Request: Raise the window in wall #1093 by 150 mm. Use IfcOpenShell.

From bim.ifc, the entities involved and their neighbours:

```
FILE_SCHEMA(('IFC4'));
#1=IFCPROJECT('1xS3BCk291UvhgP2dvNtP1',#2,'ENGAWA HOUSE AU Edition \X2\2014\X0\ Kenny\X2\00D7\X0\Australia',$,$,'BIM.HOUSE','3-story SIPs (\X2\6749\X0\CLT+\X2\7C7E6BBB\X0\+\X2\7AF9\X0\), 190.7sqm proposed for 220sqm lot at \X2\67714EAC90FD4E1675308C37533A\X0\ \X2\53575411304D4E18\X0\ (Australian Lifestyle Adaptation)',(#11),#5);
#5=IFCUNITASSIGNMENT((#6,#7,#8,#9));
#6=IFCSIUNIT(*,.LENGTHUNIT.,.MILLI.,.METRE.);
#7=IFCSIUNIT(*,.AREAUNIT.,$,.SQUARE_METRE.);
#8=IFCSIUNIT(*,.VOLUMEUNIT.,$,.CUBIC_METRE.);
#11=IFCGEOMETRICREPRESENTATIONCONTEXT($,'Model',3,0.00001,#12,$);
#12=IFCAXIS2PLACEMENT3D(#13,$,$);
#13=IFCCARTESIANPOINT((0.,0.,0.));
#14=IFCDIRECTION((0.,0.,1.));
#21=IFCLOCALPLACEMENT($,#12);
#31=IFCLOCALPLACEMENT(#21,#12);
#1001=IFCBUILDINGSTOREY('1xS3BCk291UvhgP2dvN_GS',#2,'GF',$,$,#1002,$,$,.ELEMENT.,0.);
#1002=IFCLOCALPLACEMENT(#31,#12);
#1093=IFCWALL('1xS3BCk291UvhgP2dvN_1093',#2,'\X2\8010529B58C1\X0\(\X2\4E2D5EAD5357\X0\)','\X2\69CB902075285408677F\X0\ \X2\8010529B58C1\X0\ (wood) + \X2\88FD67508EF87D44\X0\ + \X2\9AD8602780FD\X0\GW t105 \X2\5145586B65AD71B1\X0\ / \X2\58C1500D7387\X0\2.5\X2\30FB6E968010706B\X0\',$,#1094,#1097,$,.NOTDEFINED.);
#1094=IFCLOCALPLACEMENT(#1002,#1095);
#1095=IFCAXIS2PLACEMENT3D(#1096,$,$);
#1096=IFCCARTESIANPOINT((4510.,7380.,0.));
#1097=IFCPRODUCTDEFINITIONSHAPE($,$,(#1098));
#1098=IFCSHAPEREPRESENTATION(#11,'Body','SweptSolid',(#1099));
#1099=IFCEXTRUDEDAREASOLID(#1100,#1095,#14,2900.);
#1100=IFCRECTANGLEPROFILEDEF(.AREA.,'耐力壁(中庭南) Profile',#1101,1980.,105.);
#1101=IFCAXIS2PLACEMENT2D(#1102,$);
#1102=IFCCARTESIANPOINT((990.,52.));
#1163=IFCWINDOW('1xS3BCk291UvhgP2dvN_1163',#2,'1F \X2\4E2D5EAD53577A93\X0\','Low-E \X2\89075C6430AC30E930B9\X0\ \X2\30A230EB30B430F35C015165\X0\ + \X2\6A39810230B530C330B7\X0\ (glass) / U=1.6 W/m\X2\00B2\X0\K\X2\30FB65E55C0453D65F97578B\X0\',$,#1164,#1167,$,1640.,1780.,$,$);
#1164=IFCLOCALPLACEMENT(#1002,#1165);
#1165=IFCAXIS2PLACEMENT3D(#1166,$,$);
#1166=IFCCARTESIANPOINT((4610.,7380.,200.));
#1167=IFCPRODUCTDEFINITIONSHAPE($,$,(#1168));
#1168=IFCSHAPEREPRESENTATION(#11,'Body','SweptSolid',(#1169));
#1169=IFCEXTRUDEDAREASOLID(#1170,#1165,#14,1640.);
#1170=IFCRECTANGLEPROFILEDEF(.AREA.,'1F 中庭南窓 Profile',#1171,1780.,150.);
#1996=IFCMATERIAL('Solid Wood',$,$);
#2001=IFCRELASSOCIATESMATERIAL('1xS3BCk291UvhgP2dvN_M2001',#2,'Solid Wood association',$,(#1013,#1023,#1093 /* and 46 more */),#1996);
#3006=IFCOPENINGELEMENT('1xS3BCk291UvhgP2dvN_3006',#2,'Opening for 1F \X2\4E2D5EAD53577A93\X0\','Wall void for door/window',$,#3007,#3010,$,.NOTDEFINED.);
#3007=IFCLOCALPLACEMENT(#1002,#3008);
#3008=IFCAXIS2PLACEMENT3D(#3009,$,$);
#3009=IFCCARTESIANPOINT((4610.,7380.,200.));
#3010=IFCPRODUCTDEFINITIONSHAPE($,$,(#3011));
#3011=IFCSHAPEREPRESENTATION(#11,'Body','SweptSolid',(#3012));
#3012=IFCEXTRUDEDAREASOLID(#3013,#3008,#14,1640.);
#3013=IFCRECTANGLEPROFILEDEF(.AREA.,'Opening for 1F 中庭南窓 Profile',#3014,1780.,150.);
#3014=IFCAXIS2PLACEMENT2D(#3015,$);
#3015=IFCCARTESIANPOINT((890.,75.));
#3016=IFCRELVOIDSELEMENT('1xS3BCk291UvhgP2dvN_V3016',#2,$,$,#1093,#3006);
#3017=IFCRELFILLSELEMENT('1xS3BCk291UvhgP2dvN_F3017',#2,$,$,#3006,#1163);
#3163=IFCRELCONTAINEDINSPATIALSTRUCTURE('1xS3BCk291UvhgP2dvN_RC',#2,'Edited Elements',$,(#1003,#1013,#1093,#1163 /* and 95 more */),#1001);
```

```python
import numpy as np
import ifcopenshell
import ifcopenshell.api.geometry
import ifcopenshell.util.placement
import ifcopenshell.util.unit

model = ifcopenshell.open("bim.ifc")
unit_scale = ifcopenshell.util.unit.calculate_unit_scale(model)

window = model.by_id(1163)
opening = window.FillsVoids[0].RelatingOpeningElement
dz = 0.15 / unit_scale

shift = np.array([0.0, 0.0, dz])
# The window is not placed relative to its opening, so move both.
for product in (opening, window):
    matrix = ifcopenshell.util.placement.get_local_placement(product.ObjectPlacement)
    matrix[:3, 3] += shift
    ifcopenshell.api.geometry.edit_object_placement(model, product=product, matrix=matrix, is_si=False)

print(f"moved by {dz * unit_scale:+.3f} m")

model.write("bim_updated.ifc")
```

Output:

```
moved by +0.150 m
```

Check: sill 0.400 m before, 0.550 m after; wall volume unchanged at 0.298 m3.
